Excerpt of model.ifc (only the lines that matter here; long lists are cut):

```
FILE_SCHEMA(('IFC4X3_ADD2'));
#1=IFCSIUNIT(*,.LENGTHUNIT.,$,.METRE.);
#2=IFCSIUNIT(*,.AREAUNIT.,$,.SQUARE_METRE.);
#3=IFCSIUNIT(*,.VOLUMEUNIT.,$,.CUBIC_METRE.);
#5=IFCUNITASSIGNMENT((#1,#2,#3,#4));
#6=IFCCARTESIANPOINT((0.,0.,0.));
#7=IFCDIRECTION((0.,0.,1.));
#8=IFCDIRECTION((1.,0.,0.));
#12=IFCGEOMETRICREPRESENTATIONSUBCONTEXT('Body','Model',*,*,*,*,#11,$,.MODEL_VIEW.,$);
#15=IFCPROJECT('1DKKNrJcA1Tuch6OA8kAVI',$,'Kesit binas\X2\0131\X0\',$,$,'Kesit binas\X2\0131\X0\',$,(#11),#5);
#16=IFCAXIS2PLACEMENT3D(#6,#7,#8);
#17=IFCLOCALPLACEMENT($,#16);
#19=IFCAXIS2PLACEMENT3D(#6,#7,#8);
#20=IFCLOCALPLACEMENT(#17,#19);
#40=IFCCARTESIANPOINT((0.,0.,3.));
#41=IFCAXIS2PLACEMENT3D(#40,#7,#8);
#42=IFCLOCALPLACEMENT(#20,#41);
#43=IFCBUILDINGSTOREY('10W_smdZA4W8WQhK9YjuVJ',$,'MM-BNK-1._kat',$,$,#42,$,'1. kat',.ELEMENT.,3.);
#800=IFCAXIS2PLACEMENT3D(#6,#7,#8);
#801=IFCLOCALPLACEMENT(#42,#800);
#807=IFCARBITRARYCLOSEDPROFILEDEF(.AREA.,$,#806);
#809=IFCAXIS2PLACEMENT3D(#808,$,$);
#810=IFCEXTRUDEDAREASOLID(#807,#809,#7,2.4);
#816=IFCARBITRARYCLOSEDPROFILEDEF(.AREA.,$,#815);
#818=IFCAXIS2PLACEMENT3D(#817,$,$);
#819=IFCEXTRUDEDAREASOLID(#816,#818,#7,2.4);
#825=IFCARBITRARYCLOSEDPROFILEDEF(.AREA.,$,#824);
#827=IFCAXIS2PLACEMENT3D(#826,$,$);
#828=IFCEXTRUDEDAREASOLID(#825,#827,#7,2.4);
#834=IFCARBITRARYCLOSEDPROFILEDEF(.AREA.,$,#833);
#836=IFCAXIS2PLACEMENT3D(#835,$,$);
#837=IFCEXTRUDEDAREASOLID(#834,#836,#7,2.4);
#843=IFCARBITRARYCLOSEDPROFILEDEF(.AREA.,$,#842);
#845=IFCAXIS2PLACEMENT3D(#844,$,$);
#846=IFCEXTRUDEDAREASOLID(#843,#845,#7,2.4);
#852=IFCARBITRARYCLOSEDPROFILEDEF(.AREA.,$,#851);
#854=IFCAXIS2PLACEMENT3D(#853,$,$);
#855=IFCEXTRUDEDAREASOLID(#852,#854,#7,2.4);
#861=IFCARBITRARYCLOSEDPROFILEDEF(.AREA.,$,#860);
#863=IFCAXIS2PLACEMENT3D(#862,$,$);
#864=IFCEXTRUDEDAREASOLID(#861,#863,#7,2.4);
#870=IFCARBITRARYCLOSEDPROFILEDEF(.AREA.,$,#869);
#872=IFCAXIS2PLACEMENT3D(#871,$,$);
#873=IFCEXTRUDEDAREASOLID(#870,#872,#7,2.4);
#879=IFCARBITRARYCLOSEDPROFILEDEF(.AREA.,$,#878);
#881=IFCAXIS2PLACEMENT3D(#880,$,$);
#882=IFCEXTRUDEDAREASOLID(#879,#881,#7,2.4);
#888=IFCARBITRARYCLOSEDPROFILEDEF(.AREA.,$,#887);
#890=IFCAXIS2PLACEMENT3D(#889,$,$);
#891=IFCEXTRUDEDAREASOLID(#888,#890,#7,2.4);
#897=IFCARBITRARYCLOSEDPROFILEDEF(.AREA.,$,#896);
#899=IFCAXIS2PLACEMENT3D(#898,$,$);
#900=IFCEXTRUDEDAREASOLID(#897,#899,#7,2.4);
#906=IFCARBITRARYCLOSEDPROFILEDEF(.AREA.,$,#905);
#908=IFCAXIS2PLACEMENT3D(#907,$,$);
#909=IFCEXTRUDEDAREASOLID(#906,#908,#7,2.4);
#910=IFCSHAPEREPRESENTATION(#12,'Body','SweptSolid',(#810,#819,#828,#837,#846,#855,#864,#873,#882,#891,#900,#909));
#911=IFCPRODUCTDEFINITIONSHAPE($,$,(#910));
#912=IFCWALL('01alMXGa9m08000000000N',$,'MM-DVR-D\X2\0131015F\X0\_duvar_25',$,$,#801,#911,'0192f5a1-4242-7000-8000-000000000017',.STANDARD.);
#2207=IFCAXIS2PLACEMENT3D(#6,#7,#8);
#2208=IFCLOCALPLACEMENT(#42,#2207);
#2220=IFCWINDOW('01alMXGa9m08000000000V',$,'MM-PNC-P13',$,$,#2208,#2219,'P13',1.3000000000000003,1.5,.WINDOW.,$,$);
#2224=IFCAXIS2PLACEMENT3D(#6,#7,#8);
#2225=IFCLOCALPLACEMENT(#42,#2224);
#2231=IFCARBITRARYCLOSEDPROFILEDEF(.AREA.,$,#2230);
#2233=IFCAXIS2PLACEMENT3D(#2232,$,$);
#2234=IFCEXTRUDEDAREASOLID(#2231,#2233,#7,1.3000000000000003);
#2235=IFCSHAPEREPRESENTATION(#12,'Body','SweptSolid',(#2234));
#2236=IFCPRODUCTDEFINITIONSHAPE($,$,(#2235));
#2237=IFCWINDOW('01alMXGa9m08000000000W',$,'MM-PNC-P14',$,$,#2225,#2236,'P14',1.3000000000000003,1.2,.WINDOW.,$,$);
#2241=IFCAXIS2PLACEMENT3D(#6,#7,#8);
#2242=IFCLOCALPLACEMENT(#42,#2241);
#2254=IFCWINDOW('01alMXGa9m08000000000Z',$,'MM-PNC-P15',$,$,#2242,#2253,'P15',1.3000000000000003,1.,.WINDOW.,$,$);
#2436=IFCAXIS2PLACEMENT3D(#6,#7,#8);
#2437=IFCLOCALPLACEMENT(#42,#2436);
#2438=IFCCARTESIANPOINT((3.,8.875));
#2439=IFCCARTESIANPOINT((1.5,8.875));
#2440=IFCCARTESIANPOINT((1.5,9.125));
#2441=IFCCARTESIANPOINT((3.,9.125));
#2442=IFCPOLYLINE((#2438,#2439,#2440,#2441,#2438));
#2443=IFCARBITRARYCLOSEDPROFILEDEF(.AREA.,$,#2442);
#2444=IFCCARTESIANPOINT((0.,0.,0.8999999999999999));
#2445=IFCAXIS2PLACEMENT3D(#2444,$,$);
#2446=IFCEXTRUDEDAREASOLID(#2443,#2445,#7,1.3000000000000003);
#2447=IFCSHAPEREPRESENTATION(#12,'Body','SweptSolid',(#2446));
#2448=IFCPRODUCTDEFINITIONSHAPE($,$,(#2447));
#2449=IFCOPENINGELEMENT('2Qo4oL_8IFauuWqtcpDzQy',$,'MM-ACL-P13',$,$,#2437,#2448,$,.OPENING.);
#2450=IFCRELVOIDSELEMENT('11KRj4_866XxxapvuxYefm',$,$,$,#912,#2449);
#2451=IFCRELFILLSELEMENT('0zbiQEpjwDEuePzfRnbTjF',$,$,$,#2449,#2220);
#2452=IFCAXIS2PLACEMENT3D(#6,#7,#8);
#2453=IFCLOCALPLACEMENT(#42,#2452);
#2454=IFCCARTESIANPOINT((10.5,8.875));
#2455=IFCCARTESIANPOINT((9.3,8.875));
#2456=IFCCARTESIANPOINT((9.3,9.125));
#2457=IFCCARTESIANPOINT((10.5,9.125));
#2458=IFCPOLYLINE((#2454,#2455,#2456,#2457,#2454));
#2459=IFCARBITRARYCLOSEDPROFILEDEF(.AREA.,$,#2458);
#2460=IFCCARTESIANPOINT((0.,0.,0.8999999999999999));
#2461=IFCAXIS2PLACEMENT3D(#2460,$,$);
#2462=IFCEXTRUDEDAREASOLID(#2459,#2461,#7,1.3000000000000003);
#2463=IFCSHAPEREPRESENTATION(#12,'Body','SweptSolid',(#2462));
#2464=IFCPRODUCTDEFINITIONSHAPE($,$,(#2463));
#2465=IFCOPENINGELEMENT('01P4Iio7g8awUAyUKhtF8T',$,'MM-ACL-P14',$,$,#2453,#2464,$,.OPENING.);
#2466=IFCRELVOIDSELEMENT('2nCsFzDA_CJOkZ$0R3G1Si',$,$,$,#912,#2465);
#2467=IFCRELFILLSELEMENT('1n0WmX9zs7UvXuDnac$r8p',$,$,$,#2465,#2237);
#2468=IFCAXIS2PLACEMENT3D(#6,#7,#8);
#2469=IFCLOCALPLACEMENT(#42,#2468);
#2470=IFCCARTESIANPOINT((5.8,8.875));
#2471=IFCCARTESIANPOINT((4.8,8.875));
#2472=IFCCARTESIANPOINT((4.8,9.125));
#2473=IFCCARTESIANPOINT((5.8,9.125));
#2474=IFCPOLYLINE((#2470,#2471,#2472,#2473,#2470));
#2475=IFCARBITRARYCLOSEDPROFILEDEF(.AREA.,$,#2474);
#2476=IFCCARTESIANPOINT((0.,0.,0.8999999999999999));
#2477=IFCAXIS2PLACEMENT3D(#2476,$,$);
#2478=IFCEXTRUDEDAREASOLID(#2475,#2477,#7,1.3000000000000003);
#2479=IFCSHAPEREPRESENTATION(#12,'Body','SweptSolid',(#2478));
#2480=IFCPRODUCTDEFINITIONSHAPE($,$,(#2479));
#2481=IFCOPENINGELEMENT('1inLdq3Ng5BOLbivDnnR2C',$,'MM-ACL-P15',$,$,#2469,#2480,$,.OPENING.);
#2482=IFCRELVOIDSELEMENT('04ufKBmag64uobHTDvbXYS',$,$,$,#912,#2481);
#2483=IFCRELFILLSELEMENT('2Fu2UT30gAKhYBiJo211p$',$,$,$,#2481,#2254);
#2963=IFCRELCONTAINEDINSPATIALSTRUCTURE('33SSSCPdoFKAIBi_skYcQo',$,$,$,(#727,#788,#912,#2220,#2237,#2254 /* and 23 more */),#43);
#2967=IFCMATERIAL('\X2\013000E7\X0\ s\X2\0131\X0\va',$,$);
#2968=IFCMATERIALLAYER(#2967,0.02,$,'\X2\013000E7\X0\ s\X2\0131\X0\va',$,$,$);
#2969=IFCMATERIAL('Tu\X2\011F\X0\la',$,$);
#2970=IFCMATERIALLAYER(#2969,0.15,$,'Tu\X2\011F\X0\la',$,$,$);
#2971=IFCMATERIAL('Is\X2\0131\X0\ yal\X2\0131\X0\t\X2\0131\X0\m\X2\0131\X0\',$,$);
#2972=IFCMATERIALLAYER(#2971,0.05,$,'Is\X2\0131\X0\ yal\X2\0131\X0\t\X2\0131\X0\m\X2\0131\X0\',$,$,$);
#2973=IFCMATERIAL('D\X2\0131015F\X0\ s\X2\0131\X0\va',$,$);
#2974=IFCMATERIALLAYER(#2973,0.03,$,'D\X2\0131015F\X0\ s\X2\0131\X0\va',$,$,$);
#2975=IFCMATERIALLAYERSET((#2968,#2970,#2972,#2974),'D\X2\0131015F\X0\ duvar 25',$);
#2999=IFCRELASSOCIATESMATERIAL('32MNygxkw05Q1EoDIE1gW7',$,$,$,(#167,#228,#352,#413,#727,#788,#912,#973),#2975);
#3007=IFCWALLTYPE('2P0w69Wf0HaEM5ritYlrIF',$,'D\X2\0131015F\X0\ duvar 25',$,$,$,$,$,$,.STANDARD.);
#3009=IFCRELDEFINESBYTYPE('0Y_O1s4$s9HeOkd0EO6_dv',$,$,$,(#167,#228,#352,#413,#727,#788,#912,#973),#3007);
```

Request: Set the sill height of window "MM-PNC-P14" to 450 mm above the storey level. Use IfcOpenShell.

```python
import numpy as np
import ifcopenshell
import ifcopenshell.api.geometry
import ifcopenshell.geom
import ifcopenshell.util.element
import ifcopenshell.util.placement
import ifcopenshell.util.shape
import ifcopenshell.util.unit

model = ifcopenshell.open("model.ifc")
unit_scale = ifcopenshell.util.unit.calculate_unit_scale(model)

window = model.by_id(2237)
opening = window.FillsVoids[0].RelatingOpeningElement
storey = ifcopenshell.util.element.get_container(window, ifc_class="IfcBuildingStorey")
level = ifcopenshell.util.placement.get_local_placement(storey.ObjectPlacement)[2, 3]

# The opening's origin need not be at the sill, so measure its lowest point.
shape = ifcopenshell.geom.create_shape(ifcopenshell.geom.settings(), opening)
bottom = ifcopenshell.util.shape.get_shape_bottom_elevation(shape, shape.geometry) / unit_scale
dz = level + 0.45 - bottom

shift = np.array([0.0, 0.0, dz])
# The window is not placed relative to its opening, so move both.
for product in (opening, window):
    matrix = ifcopenshell.util.placement.get_local_placement(product.ObjectPlacement)
    matrix[:3, 3] += shift
    ifcopenshell.api.geometry.edit_object_placement(model, product=product, matrix=matrix, is_si=False)

print(f"moved by {dz * unit_scale:+.3f} m")

model.write("model_edited.ifc")
```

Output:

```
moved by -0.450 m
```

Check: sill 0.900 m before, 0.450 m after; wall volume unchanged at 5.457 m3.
